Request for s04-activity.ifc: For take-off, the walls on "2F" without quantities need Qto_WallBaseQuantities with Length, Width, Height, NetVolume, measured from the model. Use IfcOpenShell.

First a look at what the model holds.

```python
import ifcopenshell
import ifcopenshell.util.element
import ifcopenshell.util.unit

model = ifcopenshell.open("s04-activity.ifc")
print(model.schema)
for unit_type in ("LENGTHUNIT", "AREAUNIT", "VOLUMEUNIT"):
    print(unit_type, ifcopenshell.util.unit.calculate_unit_scale(model, unit_type))
storey = next(s for s in model.by_type("IfcBuildingStorey") if s.Name == "2F")
walls = [e for e in ifcopenshell.util.element.get_decomposition(storey) if e.is_a("IfcWall")]
for e in sorted(walls, key=lambda e: e.id()):
    print(e.id(), e.is_a(), e.Name, list(ifcopenshell.util.element.get_psets(e, qtos_only=True)), sep=" | ")
```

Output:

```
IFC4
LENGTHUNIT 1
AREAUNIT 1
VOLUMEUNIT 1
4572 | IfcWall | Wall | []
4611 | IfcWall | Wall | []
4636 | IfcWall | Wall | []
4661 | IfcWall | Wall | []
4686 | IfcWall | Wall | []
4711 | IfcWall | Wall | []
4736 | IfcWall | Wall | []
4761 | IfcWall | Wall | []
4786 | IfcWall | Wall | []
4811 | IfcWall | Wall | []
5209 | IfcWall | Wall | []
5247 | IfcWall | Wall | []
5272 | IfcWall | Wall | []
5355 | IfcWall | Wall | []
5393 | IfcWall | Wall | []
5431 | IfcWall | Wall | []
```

```python
import ifcopenshell
import ifcopenshell.api.pset
import ifcopenshell.geom
import ifcopenshell.util.element
import ifcopenshell.util.shape
import ifcopenshell.util.unit

model = ifcopenshell.open("s04-activity.ifc")
unit_scale = ifcopenshell.util.unit.calculate_unit_scale(model)
volume_scale = ifcopenshell.util.unit.calculate_unit_scale(model, "VOLUMEUNIT")
settings = ifcopenshell.geom.settings()

storey = next(s for s in model.by_type("IfcBuildingStorey") if s.Name == "2F")
walls = [e for e in ifcopenshell.util.element.get_decomposition(storey) if e.is_a("IfcWall")]

for e in sorted(walls, key=lambda e: e.id()):
    if ifcopenshell.util.element.get_psets(e, qtos_only=True, should_inherit=False):
        continue
    # Geometry comes back in metres, in the element's own axes.
    shape = ifcopenshell.geom.create_shape(settings, e)
    values = {
        "Length": ifcopenshell.util.shape.get_x(shape.geometry) / unit_scale,
        "Width": ifcopenshell.util.shape.get_y(shape.geometry) / unit_scale,
        "Height": ifcopenshell.util.shape.get_z(shape.geometry) / unit_scale,
        "NetVolume": ifcopenshell.util.shape.get_volume(shape.geometry) / volume_scale,
    }
    qto = ifcopenshell.api.pset.add_qto(model, product=e, name="Qto_WallBaseQuantities")
    ifcopenshell.api.pset.edit_qto(model, qto=qto, properties=values)
    print(e.id(), {k: round(v, 3) for k, v in values.items()})

model.write("s04-activity_edited.ifc")
```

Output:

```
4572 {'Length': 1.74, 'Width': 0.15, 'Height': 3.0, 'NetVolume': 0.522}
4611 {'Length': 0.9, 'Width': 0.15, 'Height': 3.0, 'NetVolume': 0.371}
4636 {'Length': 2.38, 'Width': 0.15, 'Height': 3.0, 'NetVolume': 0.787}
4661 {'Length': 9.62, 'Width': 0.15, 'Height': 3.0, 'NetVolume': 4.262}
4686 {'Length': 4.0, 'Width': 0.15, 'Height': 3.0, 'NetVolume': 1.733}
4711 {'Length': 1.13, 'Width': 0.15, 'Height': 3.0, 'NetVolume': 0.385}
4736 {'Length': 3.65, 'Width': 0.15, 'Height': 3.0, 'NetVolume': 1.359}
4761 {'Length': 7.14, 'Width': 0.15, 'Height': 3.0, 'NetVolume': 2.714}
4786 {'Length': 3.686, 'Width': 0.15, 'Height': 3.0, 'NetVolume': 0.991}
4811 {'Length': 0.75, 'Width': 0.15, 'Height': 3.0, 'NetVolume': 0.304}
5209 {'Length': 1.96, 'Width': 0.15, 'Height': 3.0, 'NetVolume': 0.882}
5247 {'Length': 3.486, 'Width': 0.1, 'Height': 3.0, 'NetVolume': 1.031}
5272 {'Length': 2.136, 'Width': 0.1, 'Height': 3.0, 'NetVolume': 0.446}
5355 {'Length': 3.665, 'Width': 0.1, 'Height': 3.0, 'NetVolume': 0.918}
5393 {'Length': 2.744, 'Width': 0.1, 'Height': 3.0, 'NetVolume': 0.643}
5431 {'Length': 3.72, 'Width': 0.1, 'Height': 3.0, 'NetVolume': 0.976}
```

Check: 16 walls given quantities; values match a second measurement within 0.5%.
